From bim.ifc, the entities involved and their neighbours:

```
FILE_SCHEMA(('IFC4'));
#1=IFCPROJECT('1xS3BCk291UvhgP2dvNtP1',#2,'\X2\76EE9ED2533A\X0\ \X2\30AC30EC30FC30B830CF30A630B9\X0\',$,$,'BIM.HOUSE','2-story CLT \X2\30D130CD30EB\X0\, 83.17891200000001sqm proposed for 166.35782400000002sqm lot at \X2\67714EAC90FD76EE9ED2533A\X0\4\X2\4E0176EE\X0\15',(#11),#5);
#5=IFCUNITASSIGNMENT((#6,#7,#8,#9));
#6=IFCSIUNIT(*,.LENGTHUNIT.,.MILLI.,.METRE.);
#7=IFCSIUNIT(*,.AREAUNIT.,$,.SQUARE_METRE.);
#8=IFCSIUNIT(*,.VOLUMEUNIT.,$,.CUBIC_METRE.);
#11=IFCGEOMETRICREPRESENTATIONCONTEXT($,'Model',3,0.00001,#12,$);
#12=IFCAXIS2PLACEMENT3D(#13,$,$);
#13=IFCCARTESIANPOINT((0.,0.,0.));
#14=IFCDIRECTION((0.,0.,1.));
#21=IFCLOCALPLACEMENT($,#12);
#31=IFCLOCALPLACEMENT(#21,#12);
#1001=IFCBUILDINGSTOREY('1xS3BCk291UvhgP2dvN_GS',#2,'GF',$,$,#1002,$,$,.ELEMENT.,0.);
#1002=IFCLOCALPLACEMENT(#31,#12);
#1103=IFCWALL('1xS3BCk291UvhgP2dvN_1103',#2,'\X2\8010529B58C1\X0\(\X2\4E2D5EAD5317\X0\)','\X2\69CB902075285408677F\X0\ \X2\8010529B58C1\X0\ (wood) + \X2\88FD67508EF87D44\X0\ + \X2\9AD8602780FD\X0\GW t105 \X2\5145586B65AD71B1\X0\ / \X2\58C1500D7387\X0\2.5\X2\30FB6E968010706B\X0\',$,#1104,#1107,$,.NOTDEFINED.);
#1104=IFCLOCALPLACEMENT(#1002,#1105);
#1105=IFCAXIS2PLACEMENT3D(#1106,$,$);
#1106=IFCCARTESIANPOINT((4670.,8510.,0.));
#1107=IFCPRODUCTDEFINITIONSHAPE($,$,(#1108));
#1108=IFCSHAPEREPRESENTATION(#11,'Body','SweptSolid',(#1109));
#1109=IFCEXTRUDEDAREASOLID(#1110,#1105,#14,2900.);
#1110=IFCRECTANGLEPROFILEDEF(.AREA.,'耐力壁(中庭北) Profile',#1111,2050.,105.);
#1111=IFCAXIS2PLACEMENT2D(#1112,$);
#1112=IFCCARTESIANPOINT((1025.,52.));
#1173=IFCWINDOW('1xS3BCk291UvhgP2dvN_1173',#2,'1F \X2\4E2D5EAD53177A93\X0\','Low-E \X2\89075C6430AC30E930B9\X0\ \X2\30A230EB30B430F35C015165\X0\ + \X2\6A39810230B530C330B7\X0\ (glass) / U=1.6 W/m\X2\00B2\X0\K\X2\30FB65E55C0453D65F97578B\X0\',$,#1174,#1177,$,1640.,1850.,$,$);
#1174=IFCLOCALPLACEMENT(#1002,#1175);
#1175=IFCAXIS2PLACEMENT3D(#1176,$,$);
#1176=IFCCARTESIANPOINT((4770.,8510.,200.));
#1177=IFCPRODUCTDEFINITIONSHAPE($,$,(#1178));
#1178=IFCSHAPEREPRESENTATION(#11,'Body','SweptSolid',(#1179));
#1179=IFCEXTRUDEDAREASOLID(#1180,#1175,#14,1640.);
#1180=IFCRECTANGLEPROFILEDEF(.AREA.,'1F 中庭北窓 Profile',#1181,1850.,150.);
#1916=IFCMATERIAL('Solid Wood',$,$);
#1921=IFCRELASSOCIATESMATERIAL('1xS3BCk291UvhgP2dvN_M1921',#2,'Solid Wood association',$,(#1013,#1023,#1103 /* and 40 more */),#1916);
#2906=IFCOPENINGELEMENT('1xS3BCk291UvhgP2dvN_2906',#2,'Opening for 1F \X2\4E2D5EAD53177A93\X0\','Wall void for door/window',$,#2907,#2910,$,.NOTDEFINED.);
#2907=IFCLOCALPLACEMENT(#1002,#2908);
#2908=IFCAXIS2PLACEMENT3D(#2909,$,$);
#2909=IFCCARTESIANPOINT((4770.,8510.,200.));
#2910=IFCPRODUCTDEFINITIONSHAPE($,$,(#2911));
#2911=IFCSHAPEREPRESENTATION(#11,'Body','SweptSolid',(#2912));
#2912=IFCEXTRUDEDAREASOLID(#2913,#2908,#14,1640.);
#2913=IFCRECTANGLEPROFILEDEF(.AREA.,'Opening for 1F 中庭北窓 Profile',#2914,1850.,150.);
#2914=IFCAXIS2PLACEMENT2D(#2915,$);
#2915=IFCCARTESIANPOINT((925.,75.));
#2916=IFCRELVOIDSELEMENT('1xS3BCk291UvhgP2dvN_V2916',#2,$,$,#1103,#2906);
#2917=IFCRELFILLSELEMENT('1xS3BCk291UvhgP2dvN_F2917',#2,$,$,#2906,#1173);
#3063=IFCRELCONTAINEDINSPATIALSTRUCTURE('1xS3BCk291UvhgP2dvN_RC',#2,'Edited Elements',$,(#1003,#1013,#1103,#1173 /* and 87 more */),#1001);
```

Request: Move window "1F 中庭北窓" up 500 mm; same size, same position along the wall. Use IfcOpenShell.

```python
import numpy as np
import ifcopenshell
import ifcopenshell.api.geometry
import ifcopenshell.util.placement
import ifcopenshell.util.unit

model = ifcopenshell.open("bim.ifc")
unit_scale = ifcopenshell.util.unit.calculate_unit_scale(model)

window = model.by_id(1173)
opening = window.FillsVoids[0].RelatingOpeningElement
dz = 500.0

shift = np.array([0.0, 0.0, dz])
# The window is not placed relative to its opening, so move both.
for product in (opening, window):
    matrix = ifcopenshell.util.placement.get_local_placement(product.ObjectPlacement)
    matrix[:3, 3] += shift
    ifcopenshell.api.geometry.edit_object_placement(model, product=product, matrix=matrix, is_si=False)

print(f"moved by {dz * unit_scale:+.3f} m")

model.write("bim_updated.ifc")
```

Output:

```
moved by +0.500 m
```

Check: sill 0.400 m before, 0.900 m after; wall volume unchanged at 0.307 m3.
